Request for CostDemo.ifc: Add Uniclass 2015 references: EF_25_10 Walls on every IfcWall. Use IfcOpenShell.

First a look at what the model holds.

```python
import ifcopenshell

model = ifcopenshell.open("CostDemo.ifc")
print(model.schema)
print("classifications:", [c.Name for c in model.by_type("IfcClassification")])
for ifc_class in ("IfcDoor", "IfcRoof", "IfcStair", "IfcWall", "IfcWindow"):
    print(ifc_class, len(model.by_type(ifc_class)))
```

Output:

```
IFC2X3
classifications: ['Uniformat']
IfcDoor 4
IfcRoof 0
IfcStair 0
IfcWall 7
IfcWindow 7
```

```python
import ifcopenshell
import ifcopenshell.api.classification

model = ifcopenshell.open("CostDemo.ifc")

# IFC2X3 requires Source and Edition and has no link from the project to the system.
system = model.create_entity("IfcClassification", Source="NBS", Edition="2015", Name="Uniclass 2015")

codes = {
    "IfcWall": ("EF_25_10", "Walls"),
}
for ifc_class, (code, name) in codes.items():
    products = model.by_type(ifc_class)
    ifcopenshell.api.classification.add_reference(
        model, products=products, classification=system, identification=code, name=name
    )
    print(code, len(products))

model.write("CostDemo_updated.ifc")
```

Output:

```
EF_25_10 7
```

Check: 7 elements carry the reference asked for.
